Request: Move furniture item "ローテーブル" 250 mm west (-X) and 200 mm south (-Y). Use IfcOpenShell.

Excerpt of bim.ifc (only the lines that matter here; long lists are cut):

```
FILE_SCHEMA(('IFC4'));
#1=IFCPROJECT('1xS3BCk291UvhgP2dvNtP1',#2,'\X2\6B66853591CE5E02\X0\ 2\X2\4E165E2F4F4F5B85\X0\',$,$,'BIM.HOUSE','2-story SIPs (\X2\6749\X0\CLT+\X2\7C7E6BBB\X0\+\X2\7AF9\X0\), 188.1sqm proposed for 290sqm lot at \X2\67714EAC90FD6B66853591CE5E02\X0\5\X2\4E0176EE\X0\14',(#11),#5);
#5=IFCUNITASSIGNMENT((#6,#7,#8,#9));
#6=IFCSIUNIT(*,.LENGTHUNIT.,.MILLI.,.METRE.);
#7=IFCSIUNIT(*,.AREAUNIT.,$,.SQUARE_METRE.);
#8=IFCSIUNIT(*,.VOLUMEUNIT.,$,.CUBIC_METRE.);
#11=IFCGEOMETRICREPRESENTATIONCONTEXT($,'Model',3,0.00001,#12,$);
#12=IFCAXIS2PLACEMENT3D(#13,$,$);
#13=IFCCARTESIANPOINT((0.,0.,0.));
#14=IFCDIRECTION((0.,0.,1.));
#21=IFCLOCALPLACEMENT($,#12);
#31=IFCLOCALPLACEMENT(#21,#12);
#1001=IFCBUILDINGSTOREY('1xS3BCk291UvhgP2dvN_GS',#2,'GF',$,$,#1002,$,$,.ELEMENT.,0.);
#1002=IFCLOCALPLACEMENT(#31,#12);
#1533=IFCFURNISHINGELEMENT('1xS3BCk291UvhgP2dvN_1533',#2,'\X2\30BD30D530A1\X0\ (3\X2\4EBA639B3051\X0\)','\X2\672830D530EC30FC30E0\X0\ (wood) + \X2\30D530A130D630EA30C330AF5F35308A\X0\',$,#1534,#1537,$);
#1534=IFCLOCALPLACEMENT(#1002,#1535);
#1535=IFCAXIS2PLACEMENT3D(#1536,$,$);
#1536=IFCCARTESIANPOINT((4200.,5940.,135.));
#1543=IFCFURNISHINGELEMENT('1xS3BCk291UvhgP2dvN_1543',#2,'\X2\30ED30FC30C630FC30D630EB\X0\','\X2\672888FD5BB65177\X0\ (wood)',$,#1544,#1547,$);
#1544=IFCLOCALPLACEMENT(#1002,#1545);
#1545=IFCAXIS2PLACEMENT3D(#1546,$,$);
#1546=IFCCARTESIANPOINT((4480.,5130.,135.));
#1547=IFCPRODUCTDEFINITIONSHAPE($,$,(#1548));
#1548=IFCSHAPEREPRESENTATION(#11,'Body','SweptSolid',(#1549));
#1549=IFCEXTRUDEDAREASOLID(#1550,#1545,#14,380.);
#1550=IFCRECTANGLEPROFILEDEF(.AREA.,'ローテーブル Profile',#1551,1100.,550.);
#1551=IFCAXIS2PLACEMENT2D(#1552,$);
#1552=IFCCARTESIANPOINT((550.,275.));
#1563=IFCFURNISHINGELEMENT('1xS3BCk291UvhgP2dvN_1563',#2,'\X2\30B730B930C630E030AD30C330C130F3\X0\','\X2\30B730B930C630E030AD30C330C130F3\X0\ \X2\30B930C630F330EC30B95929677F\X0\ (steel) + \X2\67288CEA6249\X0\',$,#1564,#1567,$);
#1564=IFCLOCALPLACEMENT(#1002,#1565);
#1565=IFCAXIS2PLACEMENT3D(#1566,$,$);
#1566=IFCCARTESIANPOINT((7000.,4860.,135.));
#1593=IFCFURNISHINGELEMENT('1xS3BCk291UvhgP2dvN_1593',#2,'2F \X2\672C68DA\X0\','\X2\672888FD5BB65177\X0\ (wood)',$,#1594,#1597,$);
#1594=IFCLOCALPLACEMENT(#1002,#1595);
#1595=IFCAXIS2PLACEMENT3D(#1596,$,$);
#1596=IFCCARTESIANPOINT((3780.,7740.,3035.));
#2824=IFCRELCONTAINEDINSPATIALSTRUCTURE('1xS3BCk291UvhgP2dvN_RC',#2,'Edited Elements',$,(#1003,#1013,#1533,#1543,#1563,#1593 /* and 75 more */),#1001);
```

```python
import ifcopenshell
import ifcopenshell.api.geometry
import ifcopenshell.util.placement

model = ifcopenshell.open("bim.ifc")

item = model.by_guid("1xS3BCk291UvhgP2dvN_1543")
matrix = ifcopenshell.util.placement.get_local_placement(item.ObjectPlacement)
matrix[0, 3] -= 250.0
matrix[1, 3] -= 200.0
ifcopenshell.api.geometry.edit_object_placement(model, product=item, matrix=matrix, is_si=False)

print(ifcopenshell.util.placement.get_local_placement(item.ObjectPlacement).round(3) + 0.0)

model.write("bim_edited.ifc")
```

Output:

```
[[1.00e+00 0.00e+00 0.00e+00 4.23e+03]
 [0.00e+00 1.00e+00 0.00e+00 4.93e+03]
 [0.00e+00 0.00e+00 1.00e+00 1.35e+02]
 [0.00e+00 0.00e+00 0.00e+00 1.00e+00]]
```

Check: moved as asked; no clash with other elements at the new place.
